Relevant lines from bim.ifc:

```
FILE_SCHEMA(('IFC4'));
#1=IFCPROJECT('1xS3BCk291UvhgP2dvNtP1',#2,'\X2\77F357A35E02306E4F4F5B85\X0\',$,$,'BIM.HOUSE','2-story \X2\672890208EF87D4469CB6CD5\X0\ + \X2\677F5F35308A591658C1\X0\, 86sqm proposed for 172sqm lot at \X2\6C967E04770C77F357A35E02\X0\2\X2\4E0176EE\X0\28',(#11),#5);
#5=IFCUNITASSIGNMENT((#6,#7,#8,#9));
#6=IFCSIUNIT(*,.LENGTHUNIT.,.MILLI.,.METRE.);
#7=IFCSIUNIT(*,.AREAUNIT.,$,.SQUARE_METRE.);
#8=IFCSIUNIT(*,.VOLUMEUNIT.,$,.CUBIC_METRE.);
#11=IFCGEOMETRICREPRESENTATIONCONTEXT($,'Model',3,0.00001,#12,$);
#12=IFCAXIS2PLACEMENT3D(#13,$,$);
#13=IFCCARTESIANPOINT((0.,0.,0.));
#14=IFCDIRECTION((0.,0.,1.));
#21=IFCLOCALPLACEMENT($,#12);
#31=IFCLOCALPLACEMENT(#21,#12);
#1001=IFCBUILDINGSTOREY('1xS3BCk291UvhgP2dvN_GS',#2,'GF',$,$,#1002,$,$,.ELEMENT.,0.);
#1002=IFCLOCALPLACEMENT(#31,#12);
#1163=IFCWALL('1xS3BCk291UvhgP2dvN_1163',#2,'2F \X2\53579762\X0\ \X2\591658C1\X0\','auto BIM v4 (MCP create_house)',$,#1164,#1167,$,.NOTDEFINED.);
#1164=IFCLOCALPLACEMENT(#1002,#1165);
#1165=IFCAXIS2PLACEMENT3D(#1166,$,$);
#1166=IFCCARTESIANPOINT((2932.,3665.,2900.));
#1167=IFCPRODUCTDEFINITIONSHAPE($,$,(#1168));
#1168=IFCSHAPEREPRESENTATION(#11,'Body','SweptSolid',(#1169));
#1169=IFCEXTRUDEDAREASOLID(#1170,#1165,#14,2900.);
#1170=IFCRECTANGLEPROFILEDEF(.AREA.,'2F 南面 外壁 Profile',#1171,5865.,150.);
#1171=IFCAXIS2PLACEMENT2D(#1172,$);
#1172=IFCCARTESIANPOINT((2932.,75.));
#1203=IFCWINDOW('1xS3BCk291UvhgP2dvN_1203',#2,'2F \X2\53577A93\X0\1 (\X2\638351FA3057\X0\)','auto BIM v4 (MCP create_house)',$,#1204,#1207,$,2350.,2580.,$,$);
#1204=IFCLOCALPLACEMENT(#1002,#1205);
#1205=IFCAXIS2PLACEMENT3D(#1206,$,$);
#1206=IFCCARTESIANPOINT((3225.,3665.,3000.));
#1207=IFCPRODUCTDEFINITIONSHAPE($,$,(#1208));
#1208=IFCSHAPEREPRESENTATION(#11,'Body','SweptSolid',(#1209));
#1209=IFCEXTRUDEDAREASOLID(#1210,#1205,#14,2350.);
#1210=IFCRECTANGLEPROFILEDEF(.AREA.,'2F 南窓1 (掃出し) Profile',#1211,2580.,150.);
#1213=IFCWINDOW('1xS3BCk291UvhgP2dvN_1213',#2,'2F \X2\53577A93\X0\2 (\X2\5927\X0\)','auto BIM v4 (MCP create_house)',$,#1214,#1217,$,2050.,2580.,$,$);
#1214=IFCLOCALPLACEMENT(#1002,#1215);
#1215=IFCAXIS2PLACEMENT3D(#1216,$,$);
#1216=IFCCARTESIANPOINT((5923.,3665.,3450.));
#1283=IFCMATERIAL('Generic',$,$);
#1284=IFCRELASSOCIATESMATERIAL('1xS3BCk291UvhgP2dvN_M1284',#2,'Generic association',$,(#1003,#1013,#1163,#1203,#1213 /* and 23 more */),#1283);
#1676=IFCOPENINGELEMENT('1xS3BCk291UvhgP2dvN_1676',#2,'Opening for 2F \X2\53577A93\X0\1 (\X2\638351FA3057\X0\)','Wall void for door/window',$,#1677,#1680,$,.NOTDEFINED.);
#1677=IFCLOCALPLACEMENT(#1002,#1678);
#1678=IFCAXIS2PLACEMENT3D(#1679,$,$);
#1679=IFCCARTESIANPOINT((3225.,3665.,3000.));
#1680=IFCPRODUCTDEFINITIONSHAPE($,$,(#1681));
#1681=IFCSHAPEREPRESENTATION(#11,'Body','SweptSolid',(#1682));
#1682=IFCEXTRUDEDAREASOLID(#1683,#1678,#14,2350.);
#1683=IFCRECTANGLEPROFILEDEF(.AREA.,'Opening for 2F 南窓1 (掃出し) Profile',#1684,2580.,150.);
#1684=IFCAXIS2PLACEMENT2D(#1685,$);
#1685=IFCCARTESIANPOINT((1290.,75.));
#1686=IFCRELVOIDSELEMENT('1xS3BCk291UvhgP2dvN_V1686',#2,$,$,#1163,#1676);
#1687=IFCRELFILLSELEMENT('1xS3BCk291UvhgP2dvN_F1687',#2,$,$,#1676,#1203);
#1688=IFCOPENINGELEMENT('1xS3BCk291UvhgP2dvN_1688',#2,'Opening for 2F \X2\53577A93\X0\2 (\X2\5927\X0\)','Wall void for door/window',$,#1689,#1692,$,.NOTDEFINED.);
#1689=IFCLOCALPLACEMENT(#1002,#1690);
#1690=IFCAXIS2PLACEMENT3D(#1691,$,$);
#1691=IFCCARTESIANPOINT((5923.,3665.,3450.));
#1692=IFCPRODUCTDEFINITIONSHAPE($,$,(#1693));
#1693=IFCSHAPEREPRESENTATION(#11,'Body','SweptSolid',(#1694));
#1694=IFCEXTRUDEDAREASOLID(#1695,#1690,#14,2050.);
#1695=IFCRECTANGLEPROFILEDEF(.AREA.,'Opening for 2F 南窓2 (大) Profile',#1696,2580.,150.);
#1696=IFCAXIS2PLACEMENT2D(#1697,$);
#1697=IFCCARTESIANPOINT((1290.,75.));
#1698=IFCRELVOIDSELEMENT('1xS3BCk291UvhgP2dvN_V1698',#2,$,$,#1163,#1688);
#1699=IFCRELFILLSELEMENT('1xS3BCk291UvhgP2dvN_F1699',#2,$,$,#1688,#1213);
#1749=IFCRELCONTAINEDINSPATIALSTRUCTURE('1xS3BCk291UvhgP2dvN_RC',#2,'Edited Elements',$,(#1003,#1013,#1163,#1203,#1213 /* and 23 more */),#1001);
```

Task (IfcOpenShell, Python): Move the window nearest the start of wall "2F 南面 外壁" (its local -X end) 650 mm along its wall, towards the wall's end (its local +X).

```python
import ifcopenshell
import ifcopenshell.api.geometry
import ifcopenshell.util.placement
import ifcopenshell.util.unit

model = ifcopenshell.open("bim.ifc")
unit_scale = ifcopenshell.util.unit.calculate_unit_scale(model)

window = model.by_guid("1xS3BCk291UvhgP2dvN_1203")
opening = window.FillsVoids[0].RelatingOpeningElement
wall = opening.VoidsElements[0].RelatingBuildingElement

wall_matrix = ifcopenshell.util.placement.get_local_placement(wall.ObjectPlacement)
shift = wall_matrix[:3, 0] * 0.65 / unit_scale
before = ifcopenshell.util.placement.get_local_placement(window.ObjectPlacement)[:3, 3].copy()

# The window is not placed relative to its opening, so move both.
for product in (opening, window):
    matrix = ifcopenshell.util.placement.get_local_placement(product.ObjectPlacement)
    matrix[:3, 3] += shift
    ifcopenshell.api.geometry.edit_object_placement(model, product=product, matrix=matrix, is_si=False)

after = ifcopenshell.util.placement.get_local_placement(window.ObjectPlacement)[:3, 3]
print("window moved by", (after - before).round(3) + 0.0)

model.write("bim_rev.ifc")
```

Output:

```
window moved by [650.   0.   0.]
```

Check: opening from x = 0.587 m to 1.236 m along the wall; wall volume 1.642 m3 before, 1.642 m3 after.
